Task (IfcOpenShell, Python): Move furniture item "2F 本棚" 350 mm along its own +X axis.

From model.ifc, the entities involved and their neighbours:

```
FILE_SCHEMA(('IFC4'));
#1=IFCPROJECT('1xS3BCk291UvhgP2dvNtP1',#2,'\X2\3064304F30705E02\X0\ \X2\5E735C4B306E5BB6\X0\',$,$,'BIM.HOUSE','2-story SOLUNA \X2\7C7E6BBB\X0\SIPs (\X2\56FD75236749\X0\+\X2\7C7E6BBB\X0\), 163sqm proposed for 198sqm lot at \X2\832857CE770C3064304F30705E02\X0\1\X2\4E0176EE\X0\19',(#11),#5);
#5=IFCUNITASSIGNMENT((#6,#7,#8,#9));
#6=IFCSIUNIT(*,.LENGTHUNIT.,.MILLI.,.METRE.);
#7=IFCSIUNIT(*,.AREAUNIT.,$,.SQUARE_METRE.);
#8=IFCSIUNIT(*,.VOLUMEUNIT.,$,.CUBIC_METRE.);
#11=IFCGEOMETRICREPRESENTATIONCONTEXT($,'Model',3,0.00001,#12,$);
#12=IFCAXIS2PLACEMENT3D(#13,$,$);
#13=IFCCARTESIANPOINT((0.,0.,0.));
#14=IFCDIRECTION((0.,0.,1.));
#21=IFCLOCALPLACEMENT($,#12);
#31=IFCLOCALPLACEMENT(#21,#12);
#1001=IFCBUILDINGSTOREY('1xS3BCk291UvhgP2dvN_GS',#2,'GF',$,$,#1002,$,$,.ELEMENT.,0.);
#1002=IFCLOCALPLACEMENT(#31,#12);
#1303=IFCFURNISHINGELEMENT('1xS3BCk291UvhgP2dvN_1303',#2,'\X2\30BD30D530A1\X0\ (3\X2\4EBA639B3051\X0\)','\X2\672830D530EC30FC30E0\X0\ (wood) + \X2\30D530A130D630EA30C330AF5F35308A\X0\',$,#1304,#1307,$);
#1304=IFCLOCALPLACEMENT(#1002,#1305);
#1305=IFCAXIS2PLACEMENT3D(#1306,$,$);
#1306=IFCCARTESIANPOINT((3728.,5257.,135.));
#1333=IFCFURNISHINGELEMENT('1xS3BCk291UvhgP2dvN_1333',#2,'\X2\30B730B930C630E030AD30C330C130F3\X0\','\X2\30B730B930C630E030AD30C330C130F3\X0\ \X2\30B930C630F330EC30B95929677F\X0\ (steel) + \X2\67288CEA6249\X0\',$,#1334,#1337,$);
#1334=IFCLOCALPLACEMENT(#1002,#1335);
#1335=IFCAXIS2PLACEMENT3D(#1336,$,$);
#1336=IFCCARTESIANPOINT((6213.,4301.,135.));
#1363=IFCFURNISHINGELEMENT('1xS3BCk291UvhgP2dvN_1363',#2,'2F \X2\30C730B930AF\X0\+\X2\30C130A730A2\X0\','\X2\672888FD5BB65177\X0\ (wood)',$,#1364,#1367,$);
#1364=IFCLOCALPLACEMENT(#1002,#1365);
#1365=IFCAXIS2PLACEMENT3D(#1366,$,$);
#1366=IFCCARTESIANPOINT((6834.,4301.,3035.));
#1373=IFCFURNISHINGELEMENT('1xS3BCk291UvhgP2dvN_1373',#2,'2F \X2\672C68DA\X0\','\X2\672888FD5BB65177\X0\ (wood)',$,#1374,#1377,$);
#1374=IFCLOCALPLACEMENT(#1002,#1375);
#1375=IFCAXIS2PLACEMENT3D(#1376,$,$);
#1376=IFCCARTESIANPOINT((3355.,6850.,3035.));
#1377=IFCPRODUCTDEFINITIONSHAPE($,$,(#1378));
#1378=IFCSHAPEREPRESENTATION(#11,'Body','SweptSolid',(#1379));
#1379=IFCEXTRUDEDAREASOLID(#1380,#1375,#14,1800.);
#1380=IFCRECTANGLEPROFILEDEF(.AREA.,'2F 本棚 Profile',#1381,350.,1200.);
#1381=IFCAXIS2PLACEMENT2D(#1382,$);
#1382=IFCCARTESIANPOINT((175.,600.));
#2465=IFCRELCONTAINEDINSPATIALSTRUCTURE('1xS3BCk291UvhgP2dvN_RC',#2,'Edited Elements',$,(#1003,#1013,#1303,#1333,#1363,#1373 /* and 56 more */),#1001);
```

```python
import ifcopenshell
import ifcopenshell.api.geometry
import ifcopenshell.util.placement
import ifcopenshell.util.unit

model = ifcopenshell.open("model.ifc")
unit_scale = ifcopenshell.util.unit.calculate_unit_scale(model)

item = model.by_guid("1xS3BCk291UvhgP2dvN_1373")
matrix = ifcopenshell.util.placement.get_local_placement(item.ObjectPlacement)
matrix[:3, 3] += matrix[:3, 0] * 0.35 / unit_scale
ifcopenshell.api.geometry.edit_object_placement(model, product=item, matrix=matrix, is_si=False)

print(ifcopenshell.util.placement.get_local_placement(item.ObjectPlacement).round(3) + 0.0)

model.write("model_rev.ifc")
```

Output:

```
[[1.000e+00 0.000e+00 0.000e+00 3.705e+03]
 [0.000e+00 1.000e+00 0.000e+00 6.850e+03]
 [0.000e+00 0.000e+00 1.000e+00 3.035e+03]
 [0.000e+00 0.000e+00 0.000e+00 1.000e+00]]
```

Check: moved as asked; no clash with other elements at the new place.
